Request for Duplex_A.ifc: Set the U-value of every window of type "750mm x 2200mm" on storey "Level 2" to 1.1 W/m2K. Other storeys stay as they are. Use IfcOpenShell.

First a look at what the model holds.

```python
import ifcopenshell
import ifcopenshell.util.element

model = ifcopenshell.open("Duplex_A.ifc")
print(model.schema)
storey = next(s for s in model.by_type("IfcBuildingStorey") if s.Name == "Level 2")
windows = [e for e in ifcopenshell.util.element.get_decomposition(storey) if e.is_a("IfcWindow")]
seen = {}
for e in windows:
    element_type = ifcopenshell.util.element.get_type(e)
    key = (element_type.Name if element_type != e and element_type else None, ifcopenshell.util.element.get_pset(e, "Pset_WindowCommon", "ThermalTransmittance"))
    seen[key] = seen.get(key, 0) + 1
for (name, value), count in sorted(seen.items(), key=str):
    print(count, "x", name, "|", value)
```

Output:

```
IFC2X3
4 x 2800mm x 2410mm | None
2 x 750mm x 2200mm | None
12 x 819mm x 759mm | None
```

```python
import ifcopenshell
import ifcopenshell.api.pset
import ifcopenshell.util.element

model = ifcopenshell.open("Duplex_A.ifc")

storey = next(s for s in model.by_type("IfcBuildingStorey") if s.Name == "Level 2")
windows = [e for e in ifcopenshell.util.element.get_decomposition(storey) if e.is_a("IfcWindow")]

count = 0
for e in windows:
    element_type = ifcopenshell.util.element.get_type(e)
    if element_type in (None, e) or element_type.Name != "750mm x 2200mm":
        continue
    # add_pset returns the element's existing set when there is one.
    pset = ifcopenshell.api.pset.add_pset(model, product=e, name="Pset_WindowCommon")
    ifcopenshell.api.pset.edit_pset(model, pset=pset, properties={"ThermalTransmittance": 1.1})
    count += 1

print(count, "windows updated")

model.write("Duplex_A-out.ifc")
```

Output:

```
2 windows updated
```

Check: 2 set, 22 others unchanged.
